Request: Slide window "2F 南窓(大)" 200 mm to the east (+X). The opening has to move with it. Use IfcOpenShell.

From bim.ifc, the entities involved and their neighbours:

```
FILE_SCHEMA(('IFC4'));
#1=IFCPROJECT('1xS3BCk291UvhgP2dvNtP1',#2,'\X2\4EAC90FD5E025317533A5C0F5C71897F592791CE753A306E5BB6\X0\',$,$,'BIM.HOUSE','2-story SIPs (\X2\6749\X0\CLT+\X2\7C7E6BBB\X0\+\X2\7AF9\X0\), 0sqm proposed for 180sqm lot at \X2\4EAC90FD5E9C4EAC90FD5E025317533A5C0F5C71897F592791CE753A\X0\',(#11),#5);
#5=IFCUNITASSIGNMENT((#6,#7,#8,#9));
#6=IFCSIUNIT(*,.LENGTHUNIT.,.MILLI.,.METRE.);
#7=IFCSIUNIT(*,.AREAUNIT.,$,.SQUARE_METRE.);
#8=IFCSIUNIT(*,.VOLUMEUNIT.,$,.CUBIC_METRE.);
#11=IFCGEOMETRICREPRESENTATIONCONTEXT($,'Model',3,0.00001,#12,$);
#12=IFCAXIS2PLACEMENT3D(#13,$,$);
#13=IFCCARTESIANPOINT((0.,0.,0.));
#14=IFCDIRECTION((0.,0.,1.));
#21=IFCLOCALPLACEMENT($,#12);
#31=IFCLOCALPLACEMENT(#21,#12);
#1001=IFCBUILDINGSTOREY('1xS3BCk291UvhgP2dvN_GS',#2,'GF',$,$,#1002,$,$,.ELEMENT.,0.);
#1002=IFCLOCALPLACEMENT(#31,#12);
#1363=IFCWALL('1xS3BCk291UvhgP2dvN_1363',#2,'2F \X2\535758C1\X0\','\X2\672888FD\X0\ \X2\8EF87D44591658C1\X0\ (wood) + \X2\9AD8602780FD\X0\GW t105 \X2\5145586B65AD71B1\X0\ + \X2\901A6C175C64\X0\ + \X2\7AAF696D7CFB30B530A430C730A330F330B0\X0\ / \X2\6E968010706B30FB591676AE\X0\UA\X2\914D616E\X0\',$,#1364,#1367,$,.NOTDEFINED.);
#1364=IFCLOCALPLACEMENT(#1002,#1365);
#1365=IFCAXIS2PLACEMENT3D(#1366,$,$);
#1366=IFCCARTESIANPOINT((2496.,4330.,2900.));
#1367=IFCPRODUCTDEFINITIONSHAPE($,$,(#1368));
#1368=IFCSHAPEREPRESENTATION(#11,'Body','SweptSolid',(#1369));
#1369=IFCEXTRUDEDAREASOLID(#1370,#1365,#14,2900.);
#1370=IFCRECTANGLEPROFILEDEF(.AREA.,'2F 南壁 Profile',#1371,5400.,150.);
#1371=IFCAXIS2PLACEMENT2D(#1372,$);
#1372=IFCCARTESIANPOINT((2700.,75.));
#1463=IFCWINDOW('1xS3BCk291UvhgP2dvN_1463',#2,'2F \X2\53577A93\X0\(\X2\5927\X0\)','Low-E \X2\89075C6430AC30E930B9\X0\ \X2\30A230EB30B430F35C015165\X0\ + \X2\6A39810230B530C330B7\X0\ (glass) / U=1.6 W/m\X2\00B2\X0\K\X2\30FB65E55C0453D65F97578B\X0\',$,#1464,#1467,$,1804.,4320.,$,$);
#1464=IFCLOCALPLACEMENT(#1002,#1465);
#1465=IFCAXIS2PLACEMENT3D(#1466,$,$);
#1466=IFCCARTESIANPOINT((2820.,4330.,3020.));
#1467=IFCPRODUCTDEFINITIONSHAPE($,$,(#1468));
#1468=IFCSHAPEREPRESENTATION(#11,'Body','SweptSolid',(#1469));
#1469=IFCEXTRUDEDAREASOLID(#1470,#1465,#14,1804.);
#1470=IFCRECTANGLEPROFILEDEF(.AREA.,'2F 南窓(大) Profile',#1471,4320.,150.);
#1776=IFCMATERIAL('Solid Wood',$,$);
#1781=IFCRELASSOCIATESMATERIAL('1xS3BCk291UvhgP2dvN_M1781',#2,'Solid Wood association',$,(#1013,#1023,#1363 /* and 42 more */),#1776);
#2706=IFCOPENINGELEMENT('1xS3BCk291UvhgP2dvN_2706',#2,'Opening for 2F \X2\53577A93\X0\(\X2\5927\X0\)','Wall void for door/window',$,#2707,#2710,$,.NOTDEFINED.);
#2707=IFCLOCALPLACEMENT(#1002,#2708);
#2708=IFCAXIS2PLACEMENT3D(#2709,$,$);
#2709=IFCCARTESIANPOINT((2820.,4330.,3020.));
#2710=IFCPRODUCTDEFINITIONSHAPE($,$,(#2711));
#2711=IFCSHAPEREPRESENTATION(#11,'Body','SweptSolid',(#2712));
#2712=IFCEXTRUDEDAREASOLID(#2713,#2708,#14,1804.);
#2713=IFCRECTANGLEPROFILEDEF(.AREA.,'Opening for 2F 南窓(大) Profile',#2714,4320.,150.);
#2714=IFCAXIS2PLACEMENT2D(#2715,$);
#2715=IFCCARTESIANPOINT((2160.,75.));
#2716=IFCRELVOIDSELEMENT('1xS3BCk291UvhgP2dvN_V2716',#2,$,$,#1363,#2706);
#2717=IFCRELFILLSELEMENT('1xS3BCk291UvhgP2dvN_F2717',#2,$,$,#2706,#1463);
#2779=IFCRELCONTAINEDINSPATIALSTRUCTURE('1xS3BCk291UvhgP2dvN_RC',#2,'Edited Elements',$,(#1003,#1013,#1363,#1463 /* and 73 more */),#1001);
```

```python
import ifcopenshell
import ifcopenshell.api.geometry
import ifcopenshell.util.placement

model = ifcopenshell.open("bim.ifc")

window = model.by_guid("1xS3BCk291UvhgP2dvN_1463")
opening = window.FillsVoids[0].RelatingOpeningElement
wall = opening.VoidsElements[0].RelatingBuildingElement

wall_matrix = ifcopenshell.util.placement.get_local_placement(wall.ObjectPlacement)
shift = wall_matrix[:3, 0] * 200.0
before = ifcopenshell.util.placement.get_local_placement(window.ObjectPlacement)[:3, 3].copy()

# The window is not placed relative to its opening, so move both.
for product in (opening, window):
    matrix = ifcopenshell.util.placement.get_local_placement(product.ObjectPlacement)
    matrix[:3, 3] += shift
    ifcopenshell.api.geometry.edit_object_placement(model, product=product, matrix=matrix, is_si=False)

after = ifcopenshell.util.placement.get_local_placement(window.ObjectPlacement)[:3, 3]
print("window moved by", (after - before).round(3) + 0.0)

model.write("bim_rev.ifc")
```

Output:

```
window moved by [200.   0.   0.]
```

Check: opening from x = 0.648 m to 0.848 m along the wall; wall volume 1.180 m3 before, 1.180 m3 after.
